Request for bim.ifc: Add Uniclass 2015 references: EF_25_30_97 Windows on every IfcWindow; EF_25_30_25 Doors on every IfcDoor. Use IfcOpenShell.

First a look at what the model holds.

```python
import ifcopenshell

model = ifcopenshell.open("bim.ifc")
print(model.schema)
print("classifications:", [c.Name for c in model.by_type("IfcClassification")])
for ifc_class in ("IfcDoor", "IfcRoof", "IfcStair", "IfcWall", "IfcWindow"):
    print(ifc_class, len(model.by_type(ifc_class)))
```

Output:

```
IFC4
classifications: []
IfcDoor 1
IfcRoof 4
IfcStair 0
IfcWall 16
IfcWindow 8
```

```python
import ifcopenshell
import ifcopenshell.api.classification

model = ifcopenshell.open("bim.ifc")

system = ifcopenshell.api.classification.add_classification(model, classification="Uniclass 2015")

codes = {
    "IfcWindow": ("EF_25_30_97", "Windows"),
    "IfcDoor": ("EF_25_30_25", "Doors"),
}
for ifc_class, (code, name) in codes.items():
    products = model.by_type(ifc_class)
    ifcopenshell.api.classification.add_reference(
        model, products=products, classification=system, identification=code, name=name
    )
    print(code, len(products))

model.write("bim_rev.ifc")
```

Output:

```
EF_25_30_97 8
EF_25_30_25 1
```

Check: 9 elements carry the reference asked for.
